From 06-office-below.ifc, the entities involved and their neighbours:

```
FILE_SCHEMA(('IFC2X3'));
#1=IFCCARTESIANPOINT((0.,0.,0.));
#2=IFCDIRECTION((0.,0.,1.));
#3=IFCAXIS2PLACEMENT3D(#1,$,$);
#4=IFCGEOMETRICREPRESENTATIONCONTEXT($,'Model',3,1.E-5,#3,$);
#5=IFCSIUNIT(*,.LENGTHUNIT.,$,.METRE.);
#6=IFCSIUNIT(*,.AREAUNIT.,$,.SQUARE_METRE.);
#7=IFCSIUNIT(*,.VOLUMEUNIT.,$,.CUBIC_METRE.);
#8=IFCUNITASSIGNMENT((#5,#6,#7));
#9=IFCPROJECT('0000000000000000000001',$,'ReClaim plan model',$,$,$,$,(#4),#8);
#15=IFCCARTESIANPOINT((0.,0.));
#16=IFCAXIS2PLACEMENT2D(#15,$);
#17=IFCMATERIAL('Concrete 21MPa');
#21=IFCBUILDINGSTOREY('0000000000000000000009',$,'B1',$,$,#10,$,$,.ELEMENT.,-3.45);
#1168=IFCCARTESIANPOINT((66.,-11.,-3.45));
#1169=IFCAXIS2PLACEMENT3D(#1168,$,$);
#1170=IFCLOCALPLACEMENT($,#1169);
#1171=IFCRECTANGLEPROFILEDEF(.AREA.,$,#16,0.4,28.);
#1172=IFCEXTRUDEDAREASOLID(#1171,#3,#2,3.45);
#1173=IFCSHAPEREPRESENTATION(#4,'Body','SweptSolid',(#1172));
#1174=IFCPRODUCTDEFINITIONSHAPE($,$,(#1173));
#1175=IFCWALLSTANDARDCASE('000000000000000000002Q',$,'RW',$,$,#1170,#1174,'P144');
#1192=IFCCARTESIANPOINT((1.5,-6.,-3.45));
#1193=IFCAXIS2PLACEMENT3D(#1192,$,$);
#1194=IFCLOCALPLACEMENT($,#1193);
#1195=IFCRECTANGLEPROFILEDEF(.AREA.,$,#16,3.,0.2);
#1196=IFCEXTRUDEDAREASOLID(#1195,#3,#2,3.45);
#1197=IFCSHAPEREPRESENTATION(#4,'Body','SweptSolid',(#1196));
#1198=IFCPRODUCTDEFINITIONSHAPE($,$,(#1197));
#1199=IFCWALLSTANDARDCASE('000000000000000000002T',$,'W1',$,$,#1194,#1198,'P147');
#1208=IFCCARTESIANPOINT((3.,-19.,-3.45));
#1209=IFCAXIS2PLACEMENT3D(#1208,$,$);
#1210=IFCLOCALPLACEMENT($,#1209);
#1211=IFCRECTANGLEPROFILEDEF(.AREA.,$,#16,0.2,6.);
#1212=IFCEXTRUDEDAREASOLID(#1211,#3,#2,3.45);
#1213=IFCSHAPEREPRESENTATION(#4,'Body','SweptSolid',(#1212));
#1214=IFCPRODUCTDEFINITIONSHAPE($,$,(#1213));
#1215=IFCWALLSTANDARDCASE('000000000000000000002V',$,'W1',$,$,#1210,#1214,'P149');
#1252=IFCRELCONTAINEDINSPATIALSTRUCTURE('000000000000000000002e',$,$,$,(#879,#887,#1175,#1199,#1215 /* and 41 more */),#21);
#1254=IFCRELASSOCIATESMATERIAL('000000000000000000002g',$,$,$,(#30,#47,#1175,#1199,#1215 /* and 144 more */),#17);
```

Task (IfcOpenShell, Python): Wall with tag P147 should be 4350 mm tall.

```python
import ifcopenshell
import ifcopenshell.geom
import ifcopenshell.util.shape

model = ifcopenshell.open("06-office-below.ifc")
settings = ifcopenshell.geom.settings()


def volume(element):
    """Net volume in cubic metres, openings subtracted."""
    shape = ifcopenshell.geom.create_shape(settings, element)
    return ifcopenshell.util.shape.get_volume(shape.geometry)


wall = model.by_guid("000000000000000000002T")
before = volume(wall)

body = next(r for r in wall.Representation.Representations if r.RepresentationIdentifier == "Body")
solid = body.Items[0]
old_height = solid.Depth
solid.Depth = 4.35
after = volume(wall)

print(f"height {old_height:g} -> {solid.Depth:g}, volume {before:.3f} -> {after:.3f} m3")

model.write("06-office-below_rev.ifc")
```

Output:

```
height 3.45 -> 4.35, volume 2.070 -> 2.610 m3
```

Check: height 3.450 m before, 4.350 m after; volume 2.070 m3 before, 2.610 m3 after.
